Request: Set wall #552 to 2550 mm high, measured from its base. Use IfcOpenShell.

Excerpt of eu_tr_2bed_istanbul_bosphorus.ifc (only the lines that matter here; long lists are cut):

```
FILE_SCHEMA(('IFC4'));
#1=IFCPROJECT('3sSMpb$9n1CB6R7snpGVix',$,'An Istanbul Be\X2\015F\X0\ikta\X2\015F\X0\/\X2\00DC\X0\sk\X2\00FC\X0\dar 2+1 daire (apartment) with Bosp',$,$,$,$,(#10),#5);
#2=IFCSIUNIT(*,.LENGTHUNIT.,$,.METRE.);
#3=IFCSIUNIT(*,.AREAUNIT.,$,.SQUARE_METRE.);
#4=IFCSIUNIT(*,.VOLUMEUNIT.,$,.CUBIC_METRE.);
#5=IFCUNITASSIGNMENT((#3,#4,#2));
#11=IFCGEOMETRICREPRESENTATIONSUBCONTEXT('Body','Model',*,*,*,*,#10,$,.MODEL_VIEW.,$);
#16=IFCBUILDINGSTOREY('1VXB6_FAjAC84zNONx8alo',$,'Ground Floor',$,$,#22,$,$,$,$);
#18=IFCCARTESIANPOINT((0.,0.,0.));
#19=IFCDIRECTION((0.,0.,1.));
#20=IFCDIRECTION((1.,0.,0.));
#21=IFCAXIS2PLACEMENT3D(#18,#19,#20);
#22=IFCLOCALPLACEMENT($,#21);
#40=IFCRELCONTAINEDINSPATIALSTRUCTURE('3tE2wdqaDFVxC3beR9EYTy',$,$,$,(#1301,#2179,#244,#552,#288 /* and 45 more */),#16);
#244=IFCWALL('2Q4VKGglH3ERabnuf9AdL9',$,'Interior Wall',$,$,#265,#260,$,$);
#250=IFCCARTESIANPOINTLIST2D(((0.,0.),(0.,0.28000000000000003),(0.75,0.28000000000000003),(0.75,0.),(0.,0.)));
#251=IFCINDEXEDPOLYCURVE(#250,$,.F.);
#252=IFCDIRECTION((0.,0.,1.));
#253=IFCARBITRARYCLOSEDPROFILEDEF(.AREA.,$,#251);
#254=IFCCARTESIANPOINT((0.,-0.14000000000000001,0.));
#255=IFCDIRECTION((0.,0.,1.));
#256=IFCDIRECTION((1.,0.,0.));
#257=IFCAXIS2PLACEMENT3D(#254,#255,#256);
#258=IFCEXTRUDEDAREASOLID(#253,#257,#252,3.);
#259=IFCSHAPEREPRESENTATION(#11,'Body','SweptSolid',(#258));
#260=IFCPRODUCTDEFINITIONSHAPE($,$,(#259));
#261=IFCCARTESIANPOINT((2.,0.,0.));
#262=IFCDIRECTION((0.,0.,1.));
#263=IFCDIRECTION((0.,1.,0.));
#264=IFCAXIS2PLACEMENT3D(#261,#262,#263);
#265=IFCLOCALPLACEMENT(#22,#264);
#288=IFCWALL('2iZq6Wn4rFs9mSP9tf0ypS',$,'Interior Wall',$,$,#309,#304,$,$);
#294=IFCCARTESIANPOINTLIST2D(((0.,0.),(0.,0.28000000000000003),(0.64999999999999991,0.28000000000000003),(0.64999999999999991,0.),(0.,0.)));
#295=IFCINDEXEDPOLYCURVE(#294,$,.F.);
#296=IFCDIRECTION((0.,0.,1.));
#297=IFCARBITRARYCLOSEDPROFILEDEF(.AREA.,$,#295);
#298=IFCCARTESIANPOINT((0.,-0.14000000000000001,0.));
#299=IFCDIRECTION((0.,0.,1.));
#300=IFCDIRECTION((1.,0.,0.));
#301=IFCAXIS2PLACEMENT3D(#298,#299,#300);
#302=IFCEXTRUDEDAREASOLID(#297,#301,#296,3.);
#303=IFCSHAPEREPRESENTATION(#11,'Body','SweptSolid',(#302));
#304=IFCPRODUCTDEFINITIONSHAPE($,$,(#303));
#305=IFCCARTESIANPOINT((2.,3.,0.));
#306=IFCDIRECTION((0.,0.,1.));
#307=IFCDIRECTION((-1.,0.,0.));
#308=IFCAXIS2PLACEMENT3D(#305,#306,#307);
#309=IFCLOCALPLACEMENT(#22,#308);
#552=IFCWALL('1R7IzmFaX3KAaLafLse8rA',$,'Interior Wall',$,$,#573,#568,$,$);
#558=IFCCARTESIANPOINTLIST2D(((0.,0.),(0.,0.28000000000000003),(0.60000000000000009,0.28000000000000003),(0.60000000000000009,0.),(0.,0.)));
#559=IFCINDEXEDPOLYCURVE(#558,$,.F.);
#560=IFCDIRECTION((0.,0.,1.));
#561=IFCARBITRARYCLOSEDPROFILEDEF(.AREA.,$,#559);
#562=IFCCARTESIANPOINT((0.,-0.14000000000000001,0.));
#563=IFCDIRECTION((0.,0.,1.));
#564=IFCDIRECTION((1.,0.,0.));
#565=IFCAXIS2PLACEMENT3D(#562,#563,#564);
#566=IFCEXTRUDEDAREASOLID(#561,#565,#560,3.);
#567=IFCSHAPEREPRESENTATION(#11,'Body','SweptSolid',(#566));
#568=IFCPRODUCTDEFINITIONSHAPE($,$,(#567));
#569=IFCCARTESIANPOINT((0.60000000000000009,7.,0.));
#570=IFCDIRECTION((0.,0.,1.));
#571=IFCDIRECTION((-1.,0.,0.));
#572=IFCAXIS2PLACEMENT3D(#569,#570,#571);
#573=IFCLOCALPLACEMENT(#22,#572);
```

```python
import ifcopenshell
import ifcopenshell.geom
import ifcopenshell.util.representation
import ifcopenshell.util.shape
import ifcopenshell.util.unit

model = ifcopenshell.open("eu_tr_2bed_istanbul_bosphorus.ifc")
unit_scale = ifcopenshell.util.unit.calculate_unit_scale(model)
settings = ifcopenshell.geom.settings()


def volume(element):
    """Net volume in cubic metres, openings subtracted."""
    shape = ifcopenshell.geom.create_shape(settings, element)
    return ifcopenshell.util.shape.get_volume(shape.geometry)


wall = model.by_guid("1R7IzmFaX3KAaLafLse8rA")
before = volume(wall)

body = ifcopenshell.util.representation.get_representation(wall, "Model", "Body")
solid = body.Items[0]
old_height = solid.Depth
solid.Depth = 2.55 / unit_scale
after = volume(wall)

print(f"height {old_height:g} -> {solid.Depth:g}, volume {before:.3f} -> {after:.3f} m3")

model.write("eu_tr_2bed_istanbul_bosphorus_rev.ifc")
```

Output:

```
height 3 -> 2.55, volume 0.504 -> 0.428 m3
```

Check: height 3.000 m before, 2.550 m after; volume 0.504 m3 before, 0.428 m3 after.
